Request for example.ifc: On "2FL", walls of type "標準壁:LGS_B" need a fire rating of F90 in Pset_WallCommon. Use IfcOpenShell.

First a look at what the model holds.

```python
import ifcopenshell
import ifcopenshell.util.element

model = ifcopenshell.open("example.ifc")
print(model.schema)
storey = next(s for s in model.by_type("IfcBuildingStorey") if s.Name == "2FL")
walls = [e for e in ifcopenshell.util.element.get_decomposition(storey) if e.is_a("IfcWall")]
seen = {}
for e in walls:
    element_type = ifcopenshell.util.element.get_type(e)
    key = (element_type.Name if element_type != e and element_type else None, ifcopenshell.util.element.get_pset(e, "Pset_WallCommon", "FireRating"))
    seen[key] = seen.get(key, 0) + 1
for (name, value), count in sorted(seen.items(), key=str):
    print(count, "x", name, "|", value)
```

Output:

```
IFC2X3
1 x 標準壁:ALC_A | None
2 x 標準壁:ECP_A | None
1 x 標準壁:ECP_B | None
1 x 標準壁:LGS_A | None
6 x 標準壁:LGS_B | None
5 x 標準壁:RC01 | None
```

```python
import ifcopenshell
import ifcopenshell.api.pset
import ifcopenshell.util.element

model = ifcopenshell.open("example.ifc")

storey = next(s for s in model.by_type("IfcBuildingStorey") if s.Name == "2FL")
walls = [e for e in ifcopenshell.util.element.get_decomposition(storey) if e.is_a("IfcWall")]

count = 0
for e in walls:
    element_type = ifcopenshell.util.element.get_type(e)
    if element_type in (None, e) or element_type.Name != "標準壁:LGS_B":
        continue
    # add_pset returns the element's existing set when there is one.
    pset = ifcopenshell.api.pset.add_pset(model, product=e, name="Pset_WallCommon")
    ifcopenshell.api.pset.edit_pset(model, pset=pset, properties={"FireRating": "F90"})
    count += 1

print(count, "walls updated")

model.write("example_updated.ifc")
```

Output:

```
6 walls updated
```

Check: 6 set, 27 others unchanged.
